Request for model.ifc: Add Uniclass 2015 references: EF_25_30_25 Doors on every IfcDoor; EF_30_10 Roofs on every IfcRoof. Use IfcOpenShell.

First a look at what the model holds.

```python
import ifcopenshell

model = ifcopenshell.open("model.ifc")
print(model.schema)
print("classifications:", [c.Name for c in model.by_type("IfcClassification")])
for ifc_class in ("IfcDoor", "IfcRoof", "IfcStair", "IfcWall", "IfcWindow"):
    print(ifc_class, len(model.by_type(ifc_class)))
```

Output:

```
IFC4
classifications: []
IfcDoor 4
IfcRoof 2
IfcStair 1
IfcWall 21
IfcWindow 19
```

```python
import ifcopenshell
import ifcopenshell.api.classification

model = ifcopenshell.open("model.ifc")

system = ifcopenshell.api.classification.add_classification(model, classification="Uniclass 2015")

codes = {
    "IfcDoor": ("EF_25_30_25", "Doors"),
    "IfcRoof": ("EF_30_10", "Roofs"),
}
for ifc_class, (code, name) in codes.items():
    products = model.by_type(ifc_class)
    ifcopenshell.api.classification.add_reference(
        model, products=products, classification=system, identification=code, name=name
    )
    print(code, len(products))

model.write("model-out.ifc")
```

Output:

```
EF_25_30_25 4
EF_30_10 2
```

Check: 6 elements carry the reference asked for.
